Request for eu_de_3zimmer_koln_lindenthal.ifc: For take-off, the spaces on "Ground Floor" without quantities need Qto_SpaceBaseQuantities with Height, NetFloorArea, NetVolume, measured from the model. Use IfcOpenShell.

First a look at what the model holds.

```python
import ifcopenshell
import ifcopenshell.util.element
import ifcopenshell.util.unit

model = ifcopenshell.open("eu_de_3zimmer_koln_lindenthal.ifc")
print(model.schema)
for unit_type in ("LENGTHUNIT", "AREAUNIT", "VOLUMEUNIT"):
    print(unit_type, ifcopenshell.util.unit.calculate_unit_scale(model, unit_type))
storey = next(s for s in model.by_type("IfcBuildingStorey") if s.Name == "Ground Floor")
spaces = [e for e in ifcopenshell.util.element.get_decomposition(storey) if e.is_a("IfcSpace")]
for e in sorted(spaces, key=lambda e: e.id()):
    print(e.id(), e.is_a(), e.Name, list(ifcopenshell.util.element.get_psets(e, qtos_only=True)), sep=" | ")
```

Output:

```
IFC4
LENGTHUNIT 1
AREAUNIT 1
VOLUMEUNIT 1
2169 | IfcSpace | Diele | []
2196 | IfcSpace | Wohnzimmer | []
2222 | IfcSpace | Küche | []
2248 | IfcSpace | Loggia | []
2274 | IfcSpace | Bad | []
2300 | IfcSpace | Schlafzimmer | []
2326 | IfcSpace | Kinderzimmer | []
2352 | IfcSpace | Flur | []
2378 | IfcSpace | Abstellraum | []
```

```python
import ifcopenshell
import ifcopenshell.api.pset
import ifcopenshell.geom
import ifcopenshell.util.element
import ifcopenshell.util.shape
import ifcopenshell.util.unit

model = ifcopenshell.open("eu_de_3zimmer_koln_lindenthal.ifc")
unit_scale = ifcopenshell.util.unit.calculate_unit_scale(model)
area_scale = ifcopenshell.util.unit.calculate_unit_scale(model, "AREAUNIT")
volume_scale = ifcopenshell.util.unit.calculate_unit_scale(model, "VOLUMEUNIT")
settings = ifcopenshell.geom.settings()

storey = next(s for s in model.by_type("IfcBuildingStorey") if s.Name == "Ground Floor")
spaces = [e for e in ifcopenshell.util.element.get_decomposition(storey) if e.is_a("IfcSpace")]

for e in sorted(spaces, key=lambda e: e.id()):
    if ifcopenshell.util.element.get_psets(e, qtos_only=True, should_inherit=False):
        continue
    # Geometry comes back in metres, in the element's own axes.
    shape = ifcopenshell.geom.create_shape(settings, e)
    values = {
        "Height": ifcopenshell.util.shape.get_z(shape.geometry) / unit_scale,
        "NetFloorArea": ifcopenshell.util.shape.get_footprint_area(shape.geometry) / area_scale,
        "NetVolume": ifcopenshell.util.shape.get_volume(shape.geometry) / volume_scale,
    }
    qto = ifcopenshell.api.pset.add_qto(model, product=e, name="Qto_SpaceBaseQuantities")
    ifcopenshell.api.pset.edit_qto(model, qto=qto, properties=values)
    print(e.id(), {k: round(v, 3) for k, v in values.items()})

model.write("eu_de_3zimmer_koln_lindenthal_updated.ifc")
```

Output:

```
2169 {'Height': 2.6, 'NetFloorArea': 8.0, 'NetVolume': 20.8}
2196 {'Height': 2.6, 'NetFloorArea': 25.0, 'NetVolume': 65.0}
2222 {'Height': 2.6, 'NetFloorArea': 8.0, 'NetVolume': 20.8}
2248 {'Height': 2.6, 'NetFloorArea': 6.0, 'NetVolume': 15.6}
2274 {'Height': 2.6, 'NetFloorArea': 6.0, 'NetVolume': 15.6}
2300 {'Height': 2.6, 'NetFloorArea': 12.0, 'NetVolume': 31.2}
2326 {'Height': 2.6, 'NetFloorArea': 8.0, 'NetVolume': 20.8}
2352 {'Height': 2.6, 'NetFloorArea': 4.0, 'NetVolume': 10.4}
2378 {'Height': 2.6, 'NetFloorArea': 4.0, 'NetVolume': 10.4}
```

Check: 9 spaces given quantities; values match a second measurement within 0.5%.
